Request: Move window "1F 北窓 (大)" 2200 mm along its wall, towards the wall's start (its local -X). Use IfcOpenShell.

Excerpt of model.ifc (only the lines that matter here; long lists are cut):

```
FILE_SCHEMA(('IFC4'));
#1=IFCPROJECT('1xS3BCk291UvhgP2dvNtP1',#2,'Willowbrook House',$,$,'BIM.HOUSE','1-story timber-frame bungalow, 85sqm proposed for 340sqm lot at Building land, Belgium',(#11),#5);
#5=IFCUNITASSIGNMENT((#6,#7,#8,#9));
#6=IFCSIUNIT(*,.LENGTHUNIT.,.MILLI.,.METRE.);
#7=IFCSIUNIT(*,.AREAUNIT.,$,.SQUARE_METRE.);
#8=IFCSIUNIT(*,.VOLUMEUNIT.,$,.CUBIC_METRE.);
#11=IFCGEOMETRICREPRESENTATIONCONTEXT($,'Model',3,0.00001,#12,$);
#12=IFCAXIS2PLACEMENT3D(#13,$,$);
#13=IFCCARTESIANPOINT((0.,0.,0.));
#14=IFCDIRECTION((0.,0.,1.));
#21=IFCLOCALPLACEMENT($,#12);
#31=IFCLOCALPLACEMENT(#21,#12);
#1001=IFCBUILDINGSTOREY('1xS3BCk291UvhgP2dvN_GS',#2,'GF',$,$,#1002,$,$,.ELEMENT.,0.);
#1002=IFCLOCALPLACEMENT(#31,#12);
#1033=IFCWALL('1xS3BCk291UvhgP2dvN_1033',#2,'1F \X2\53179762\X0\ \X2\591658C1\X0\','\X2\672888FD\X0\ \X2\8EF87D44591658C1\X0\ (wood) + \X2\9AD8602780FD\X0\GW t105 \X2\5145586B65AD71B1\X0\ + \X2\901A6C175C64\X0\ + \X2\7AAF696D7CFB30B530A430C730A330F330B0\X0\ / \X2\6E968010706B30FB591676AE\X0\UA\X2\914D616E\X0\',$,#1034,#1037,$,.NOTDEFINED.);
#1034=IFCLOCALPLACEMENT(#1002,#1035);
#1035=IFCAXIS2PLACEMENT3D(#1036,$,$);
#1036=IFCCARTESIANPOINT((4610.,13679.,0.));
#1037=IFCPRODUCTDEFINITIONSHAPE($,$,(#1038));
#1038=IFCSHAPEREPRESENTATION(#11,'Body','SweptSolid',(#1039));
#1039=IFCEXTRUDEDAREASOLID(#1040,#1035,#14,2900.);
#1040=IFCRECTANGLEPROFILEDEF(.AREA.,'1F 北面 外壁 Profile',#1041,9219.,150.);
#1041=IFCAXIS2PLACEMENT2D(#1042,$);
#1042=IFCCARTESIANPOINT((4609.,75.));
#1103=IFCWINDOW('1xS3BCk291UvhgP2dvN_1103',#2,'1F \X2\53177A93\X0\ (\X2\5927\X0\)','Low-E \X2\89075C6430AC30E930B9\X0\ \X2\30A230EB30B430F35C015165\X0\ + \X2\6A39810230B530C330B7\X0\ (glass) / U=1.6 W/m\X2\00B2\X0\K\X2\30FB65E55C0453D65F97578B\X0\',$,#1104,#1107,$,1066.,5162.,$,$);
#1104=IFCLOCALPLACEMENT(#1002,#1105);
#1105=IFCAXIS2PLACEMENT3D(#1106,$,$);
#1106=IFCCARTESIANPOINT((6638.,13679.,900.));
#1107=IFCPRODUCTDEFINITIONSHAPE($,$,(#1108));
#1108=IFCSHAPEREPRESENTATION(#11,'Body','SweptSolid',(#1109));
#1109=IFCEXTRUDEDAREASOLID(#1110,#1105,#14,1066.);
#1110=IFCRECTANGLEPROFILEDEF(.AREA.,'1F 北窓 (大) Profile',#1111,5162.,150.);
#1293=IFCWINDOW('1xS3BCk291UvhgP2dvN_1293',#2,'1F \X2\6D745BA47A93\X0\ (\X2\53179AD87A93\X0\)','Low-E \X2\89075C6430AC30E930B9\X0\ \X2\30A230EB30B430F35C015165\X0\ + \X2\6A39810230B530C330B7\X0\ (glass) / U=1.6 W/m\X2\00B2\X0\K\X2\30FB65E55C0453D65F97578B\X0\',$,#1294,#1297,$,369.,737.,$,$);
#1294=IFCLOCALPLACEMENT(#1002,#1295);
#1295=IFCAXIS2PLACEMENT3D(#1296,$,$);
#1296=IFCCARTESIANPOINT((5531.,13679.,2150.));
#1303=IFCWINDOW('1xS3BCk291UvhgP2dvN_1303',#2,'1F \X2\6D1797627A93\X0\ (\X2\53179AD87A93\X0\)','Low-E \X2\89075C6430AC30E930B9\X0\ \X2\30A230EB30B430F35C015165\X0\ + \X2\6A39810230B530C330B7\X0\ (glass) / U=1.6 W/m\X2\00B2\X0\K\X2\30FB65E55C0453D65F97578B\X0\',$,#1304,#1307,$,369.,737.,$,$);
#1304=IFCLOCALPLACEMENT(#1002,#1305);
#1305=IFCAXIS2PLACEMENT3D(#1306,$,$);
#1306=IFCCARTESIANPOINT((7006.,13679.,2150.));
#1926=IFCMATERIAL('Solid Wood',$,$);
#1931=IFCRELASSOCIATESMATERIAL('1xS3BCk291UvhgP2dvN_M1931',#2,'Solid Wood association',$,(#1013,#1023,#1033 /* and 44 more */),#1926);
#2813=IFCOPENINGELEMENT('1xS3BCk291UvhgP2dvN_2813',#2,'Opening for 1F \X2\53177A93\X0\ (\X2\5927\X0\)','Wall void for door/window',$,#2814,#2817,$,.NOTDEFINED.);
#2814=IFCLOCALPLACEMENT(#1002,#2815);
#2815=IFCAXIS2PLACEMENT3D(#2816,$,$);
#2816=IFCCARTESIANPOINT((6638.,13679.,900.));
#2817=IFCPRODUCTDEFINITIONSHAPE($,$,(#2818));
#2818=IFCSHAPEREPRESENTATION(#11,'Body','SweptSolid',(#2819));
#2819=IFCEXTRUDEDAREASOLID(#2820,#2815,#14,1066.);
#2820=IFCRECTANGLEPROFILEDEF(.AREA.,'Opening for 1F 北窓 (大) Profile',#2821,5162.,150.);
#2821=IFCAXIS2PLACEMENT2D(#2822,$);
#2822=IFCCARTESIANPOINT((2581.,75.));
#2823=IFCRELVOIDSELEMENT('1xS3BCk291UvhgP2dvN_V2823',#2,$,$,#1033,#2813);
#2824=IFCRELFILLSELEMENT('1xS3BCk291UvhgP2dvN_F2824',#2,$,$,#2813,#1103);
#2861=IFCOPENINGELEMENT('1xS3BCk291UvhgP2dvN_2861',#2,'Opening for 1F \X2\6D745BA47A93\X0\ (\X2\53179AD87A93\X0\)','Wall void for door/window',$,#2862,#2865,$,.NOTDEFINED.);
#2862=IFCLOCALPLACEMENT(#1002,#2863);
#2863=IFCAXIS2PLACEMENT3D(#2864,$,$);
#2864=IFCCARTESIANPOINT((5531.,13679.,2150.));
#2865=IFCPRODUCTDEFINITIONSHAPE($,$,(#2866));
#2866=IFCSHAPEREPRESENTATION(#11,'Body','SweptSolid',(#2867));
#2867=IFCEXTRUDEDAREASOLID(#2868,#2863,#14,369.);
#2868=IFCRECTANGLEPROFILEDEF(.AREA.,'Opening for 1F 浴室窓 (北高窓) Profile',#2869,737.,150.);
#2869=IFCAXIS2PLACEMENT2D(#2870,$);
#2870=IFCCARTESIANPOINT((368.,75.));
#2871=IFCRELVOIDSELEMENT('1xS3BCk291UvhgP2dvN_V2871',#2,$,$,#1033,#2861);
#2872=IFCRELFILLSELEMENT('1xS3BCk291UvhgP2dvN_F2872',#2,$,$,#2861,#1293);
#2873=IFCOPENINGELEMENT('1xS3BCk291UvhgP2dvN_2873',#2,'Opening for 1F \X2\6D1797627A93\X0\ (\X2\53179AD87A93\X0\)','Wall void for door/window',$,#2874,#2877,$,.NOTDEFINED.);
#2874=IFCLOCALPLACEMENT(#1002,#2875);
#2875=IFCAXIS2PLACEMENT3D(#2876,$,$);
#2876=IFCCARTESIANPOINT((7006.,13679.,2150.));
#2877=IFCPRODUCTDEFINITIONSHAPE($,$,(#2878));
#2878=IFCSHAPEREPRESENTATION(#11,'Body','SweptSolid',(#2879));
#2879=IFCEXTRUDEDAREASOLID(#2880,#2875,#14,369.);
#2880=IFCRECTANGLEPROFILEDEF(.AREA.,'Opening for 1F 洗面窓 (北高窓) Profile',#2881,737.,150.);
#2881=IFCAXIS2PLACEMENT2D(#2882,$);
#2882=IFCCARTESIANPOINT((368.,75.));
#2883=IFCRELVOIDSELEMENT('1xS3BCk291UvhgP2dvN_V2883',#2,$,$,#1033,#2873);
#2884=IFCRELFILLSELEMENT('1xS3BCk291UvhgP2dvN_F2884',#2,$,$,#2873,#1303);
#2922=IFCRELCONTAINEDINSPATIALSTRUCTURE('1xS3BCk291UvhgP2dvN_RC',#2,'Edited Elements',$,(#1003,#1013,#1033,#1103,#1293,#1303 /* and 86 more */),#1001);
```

```python
import ifcopenshell
import ifcopenshell.api.geometry
import ifcopenshell.util.placement
import ifcopenshell.util.unit

model = ifcopenshell.open("model.ifc")
unit_scale = ifcopenshell.util.unit.calculate_unit_scale(model)

window = model.by_id(1103)
opening = window.FillsVoids[0].RelatingOpeningElement
wall = opening.VoidsElements[0].RelatingBuildingElement

wall_matrix = ifcopenshell.util.placement.get_local_placement(wall.ObjectPlacement)
shift = wall_matrix[:3, 0] * -2.2 / unit_scale
before = ifcopenshell.util.placement.get_local_placement(window.ObjectPlacement)[:3, 3].copy()

# The window is not placed relative to its opening, so move both.
for product in (opening, window):
    matrix = ifcopenshell.util.placement.get_local_placement(product.ObjectPlacement)
    matrix[:3, 3] += shift
    ifcopenshell.api.geometry.edit_object_placement(model, product=product, matrix=matrix, is_si=False)

after = ifcopenshell.util.placement.get_local_placement(window.ObjectPlacement)[:3, 3]
print("window moved by", (after - before).round(3) + 0.0)

model.write("model_updated.ifc")
```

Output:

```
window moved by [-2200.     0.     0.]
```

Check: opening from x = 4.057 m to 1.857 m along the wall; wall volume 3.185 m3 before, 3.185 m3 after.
